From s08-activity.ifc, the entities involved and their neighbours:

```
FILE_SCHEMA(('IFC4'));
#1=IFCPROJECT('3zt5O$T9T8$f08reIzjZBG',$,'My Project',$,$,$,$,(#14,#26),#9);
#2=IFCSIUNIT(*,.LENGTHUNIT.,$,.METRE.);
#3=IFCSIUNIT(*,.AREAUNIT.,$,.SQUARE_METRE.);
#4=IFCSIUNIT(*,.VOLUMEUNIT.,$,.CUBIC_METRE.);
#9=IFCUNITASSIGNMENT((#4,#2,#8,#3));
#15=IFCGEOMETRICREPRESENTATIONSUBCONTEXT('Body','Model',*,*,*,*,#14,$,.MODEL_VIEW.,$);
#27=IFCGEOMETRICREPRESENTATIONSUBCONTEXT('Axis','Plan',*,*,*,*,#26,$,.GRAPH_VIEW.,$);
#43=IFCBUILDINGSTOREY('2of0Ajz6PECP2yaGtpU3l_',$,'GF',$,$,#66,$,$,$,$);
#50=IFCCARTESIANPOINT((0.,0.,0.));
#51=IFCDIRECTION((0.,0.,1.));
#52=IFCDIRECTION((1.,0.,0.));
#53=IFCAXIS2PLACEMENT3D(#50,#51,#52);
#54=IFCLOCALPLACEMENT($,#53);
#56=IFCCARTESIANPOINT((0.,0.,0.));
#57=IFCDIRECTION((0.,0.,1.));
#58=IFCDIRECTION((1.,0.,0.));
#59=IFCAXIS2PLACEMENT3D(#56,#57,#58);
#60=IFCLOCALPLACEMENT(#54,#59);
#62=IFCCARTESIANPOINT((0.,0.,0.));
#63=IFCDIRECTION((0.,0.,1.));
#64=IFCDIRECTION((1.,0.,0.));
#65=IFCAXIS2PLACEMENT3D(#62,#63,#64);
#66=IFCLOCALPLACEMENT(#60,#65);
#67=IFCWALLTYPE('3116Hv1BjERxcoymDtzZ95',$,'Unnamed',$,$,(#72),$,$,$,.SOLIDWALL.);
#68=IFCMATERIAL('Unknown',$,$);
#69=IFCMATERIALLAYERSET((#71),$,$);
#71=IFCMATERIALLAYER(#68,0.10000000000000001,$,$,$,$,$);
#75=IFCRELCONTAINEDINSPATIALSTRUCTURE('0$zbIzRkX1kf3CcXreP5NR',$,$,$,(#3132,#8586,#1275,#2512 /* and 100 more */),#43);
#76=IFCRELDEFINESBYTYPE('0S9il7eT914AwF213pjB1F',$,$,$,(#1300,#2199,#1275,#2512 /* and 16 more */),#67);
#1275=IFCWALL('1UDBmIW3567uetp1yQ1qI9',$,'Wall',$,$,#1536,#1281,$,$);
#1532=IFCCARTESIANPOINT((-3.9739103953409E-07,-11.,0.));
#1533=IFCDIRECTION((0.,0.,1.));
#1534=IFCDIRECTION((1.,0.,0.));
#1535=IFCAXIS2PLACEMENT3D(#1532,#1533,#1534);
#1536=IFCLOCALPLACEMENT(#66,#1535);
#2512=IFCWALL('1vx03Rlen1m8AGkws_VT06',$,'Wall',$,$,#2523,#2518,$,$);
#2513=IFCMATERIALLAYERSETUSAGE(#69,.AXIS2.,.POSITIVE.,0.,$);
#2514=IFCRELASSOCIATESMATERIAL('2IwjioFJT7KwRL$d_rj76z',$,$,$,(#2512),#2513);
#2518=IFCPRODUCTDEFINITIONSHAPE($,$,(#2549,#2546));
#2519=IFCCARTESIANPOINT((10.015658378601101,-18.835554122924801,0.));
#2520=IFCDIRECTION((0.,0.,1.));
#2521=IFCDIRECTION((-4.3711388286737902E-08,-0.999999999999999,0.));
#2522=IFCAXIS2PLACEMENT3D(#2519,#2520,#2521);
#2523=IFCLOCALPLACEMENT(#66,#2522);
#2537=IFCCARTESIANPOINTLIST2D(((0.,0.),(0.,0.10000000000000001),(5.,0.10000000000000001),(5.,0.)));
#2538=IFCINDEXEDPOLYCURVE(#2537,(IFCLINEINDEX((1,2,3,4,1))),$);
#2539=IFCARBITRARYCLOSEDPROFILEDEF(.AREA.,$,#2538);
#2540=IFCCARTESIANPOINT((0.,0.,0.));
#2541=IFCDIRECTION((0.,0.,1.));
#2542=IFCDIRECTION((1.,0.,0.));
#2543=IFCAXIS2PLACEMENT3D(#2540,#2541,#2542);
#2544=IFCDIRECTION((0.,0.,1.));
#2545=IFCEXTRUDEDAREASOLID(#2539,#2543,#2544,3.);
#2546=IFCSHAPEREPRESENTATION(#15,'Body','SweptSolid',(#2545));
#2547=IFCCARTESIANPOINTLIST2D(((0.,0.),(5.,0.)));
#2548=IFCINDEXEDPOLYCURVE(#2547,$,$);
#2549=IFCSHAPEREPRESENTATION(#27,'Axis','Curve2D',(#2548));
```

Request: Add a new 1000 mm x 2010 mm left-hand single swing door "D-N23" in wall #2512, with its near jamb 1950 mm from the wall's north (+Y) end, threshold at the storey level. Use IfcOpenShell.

```python
import numpy as np
import ifcopenshell
import ifcopenshell.api.feature
import ifcopenshell.api.geometry
import ifcopenshell.api.root
import ifcopenshell.api.spatial
import ifcopenshell.geom
import ifcopenshell.util.element
import ifcopenshell.util.placement
import ifcopenshell.util.representation
import ifcopenshell.util.shape
import ifcopenshell.util.unit

model = ifcopenshell.open("s08-activity.ifc")
unit_scale = ifcopenshell.util.unit.calculate_unit_scale(model)
settings = ifcopenshell.geom.settings()


def volume(element):
    """Net volume in cubic metres, openings subtracted."""
    shape = ifcopenshell.geom.create_shape(settings, element)
    return ifcopenshell.util.shape.get_volume(shape.geometry)


wall = model.by_id(2512)
storey = ifcopenshell.util.element.get_container(wall, ifc_class="IfcBuildingStorey")
context = ifcopenshell.util.representation.get_context(model, "Model", "Body", "MODEL_VIEW")
before = volume(wall)

width, height, from_end, sill = 1, 2.01, 1.95, 0.0  # metres

# The wall runs along its own X axis, and the end named is its -X end.
wall_shape = ifcopenshell.geom.create_shape(settings, wall)
x, y, z = ifcopenshell.util.shape.get_vertices(wall_shape.geometry).T
start = x.min() + from_end
face, thickness = float(y.min()), float(y.max() - y.min())
wall_matrix = ifcopenshell.util.placement.get_local_placement(wall.ObjectPlacement)
level = ifcopenshell.util.placement.get_local_placement(storey.ObjectPlacement)[2, 3]


def in_wall(x, y):
    """Placement at x, y metres in the wall's axes, at sill height."""
    matrix = wall_matrix.copy()
    matrix[:, 3] = wall_matrix @ np.array([x / unit_scale, y / unit_scale, 0.0, 1.0])
    matrix[2, 3] = level + sill / unit_scale
    return matrix


# Opening: a box that overshoots both wall faces by 50 mm.
opening = ifcopenshell.api.root.create_entity(model, ifc_class="IfcOpeningElement", predefined_type="OPENING")
box = ifcopenshell.api.geometry.add_wall_representation(
    model, context=context, length=width, height=height, thickness=thickness + 0.1
)
ifcopenshell.api.geometry.assign_representation(model, product=opening, representation=box)
ifcopenshell.api.geometry.edit_object_placement(model, product=opening, matrix=in_wall(start, face - 0.05), is_si=False)
ifcopenshell.api.feature.add_feature(model, feature=opening, element=wall)

door = ifcopenshell.api.root.create_entity(model, ifc_class="IfcDoor", name="D-N23", predefined_type="DOOR")
door.OverallWidth, door.OverallHeight = width / unit_scale, height / unit_scale
door.OperationType = "SINGLE_SWING_LEFT"
body = ifcopenshell.api.geometry.add_door_representation(
    model,
    context=context,
    overall_width=door.OverallWidth,
    overall_height=door.OverallHeight,
    operation_type="SINGLE_SWING_LEFT",
    lining_properties={"LiningDepth": thickness / unit_scale, "ThresholdDepth": thickness / unit_scale},
)
ifcopenshell.api.geometry.assign_representation(model, product=door, representation=body)
ifcopenshell.api.spatial.assign_container(model, products=[door], relating_structure=storey)
ifcopenshell.api.feature.add_filling(model, opening=opening, element=door)

# The lining spans the wall, so the door starts at the wall face.
ifcopenshell.api.geometry.edit_object_placement(model, product=door, matrix=in_wall(start, face), is_si=False)

after = volume(wall)

print(f"wall volume {before:.3f} -> {after:.3f} m3")

model.write("s08-activity_updated.ifc")
```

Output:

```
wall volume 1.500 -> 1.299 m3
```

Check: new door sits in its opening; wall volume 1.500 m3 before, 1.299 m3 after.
